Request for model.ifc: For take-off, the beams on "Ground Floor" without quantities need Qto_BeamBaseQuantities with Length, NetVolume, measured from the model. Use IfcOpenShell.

First a look at what the model holds.

```python
import ifcopenshell
import ifcopenshell.util.element
import ifcopenshell.util.unit

model = ifcopenshell.open("model.ifc")
print(model.schema)
for unit_type in ("LENGTHUNIT", "AREAUNIT", "VOLUMEUNIT"):
    print(unit_type, ifcopenshell.util.unit.calculate_unit_scale(model, unit_type))
storey = next(s for s in model.by_type("IfcBuildingStorey") if s.Name == "Ground Floor")
beams = [e for e in ifcopenshell.util.element.get_decomposition(storey) if e.is_a("IfcBeam")]
for e in sorted(beams, key=lambda e: e.id()):
    print(e.id(), e.is_a(), e.Name, list(ifcopenshell.util.element.get_psets(e, qtos_only=True)), sep=" | ")
```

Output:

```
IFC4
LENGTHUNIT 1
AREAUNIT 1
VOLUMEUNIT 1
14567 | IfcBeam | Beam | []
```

```python
import ifcopenshell
import ifcopenshell.api.pset
import ifcopenshell.geom
import ifcopenshell.util.element
import ifcopenshell.util.shape
import ifcopenshell.util.unit

model = ifcopenshell.open("model.ifc")
unit_scale = ifcopenshell.util.unit.calculate_unit_scale(model)
volume_scale = ifcopenshell.util.unit.calculate_unit_scale(model, "VOLUMEUNIT")
settings = ifcopenshell.geom.settings()

storey = next(s for s in model.by_type("IfcBuildingStorey") if s.Name == "Ground Floor")
beams = [e for e in ifcopenshell.util.element.get_decomposition(storey) if e.is_a("IfcBeam")]

for e in sorted(beams, key=lambda e: e.id()):
    if ifcopenshell.util.element.get_psets(e, qtos_only=True, should_inherit=False):
        continue
    # Geometry comes back in metres, in the element's own axes.
    shape = ifcopenshell.geom.create_shape(settings, e)
    values = {
        "Length": ifcopenshell.util.shape.get_max_xyz(shape.geometry) / unit_scale,
        "NetVolume": ifcopenshell.util.shape.get_volume(shape.geometry) / volume_scale,
    }
    qto = ifcopenshell.api.pset.add_qto(model, product=e, name="Qto_BeamBaseQuantities")
    ifcopenshell.api.pset.edit_qto(model, qto=qto, properties=values)
    print(e.id(), {k: round(v, 3) for k, v in values.items()})

model.write("model_rev.ifc")
```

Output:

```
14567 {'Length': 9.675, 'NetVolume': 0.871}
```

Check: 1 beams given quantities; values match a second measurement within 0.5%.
